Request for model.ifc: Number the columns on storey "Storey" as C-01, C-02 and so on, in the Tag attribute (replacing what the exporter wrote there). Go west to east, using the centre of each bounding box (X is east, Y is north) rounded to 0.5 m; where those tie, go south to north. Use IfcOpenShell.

First a look at what the model holds.

```python
import ifcopenshell
import ifcopenshell.util.element
import ifcopenshell.util.placement

model = ifcopenshell.open("model.ifc")
print(model.schema)
storey = next(s for s in model.by_type("IfcBuildingStorey") if s.Name == "Storey")
columns = [e for e in ifcopenshell.util.element.get_decomposition(storey) if e.is_a("IfcColumn")]
for e in sorted(columns, key=lambda e: e.id()):
    origin = ifcopenshell.util.placement.get_local_placement(e.ObjectPlacement)[:3, 3]
    print(e.id(), e.Tag, e.Name, origin.round(2) + 0.0, sep=" | ")
```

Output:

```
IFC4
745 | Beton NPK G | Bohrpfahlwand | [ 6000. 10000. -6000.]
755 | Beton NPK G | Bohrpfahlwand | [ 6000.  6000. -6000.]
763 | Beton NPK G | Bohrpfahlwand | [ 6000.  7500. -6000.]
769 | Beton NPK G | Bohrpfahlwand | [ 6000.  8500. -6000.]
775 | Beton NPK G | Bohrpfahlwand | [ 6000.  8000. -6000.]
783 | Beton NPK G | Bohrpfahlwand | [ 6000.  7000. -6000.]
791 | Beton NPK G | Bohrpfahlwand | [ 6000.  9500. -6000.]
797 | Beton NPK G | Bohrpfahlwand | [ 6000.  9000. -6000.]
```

```python
import ifcopenshell
import ifcopenshell.geom
import ifcopenshell.util.element
import ifcopenshell.util.shape

model = ifcopenshell.open("model.ifc")
settings = ifcopenshell.geom.settings()
settings.set("use-world-coords", True)


def centre(element):
    shape = ifcopenshell.geom.create_shape(settings, element)
    return ifcopenshell.util.shape.get_bbox_centroid(shape.geometry)


storey = next(s for s in model.by_type("IfcBuildingStorey") if s.Name == "Storey")
columns = [e for e in ifcopenshell.util.element.get_decomposition(storey) if e.is_a("IfcColumn")]

# Insertion points can sit at a corner or the storey origin, so sort by the geometry (in metres).
centres = {e: centre(e) for e in columns}
columns.sort(key=lambda e: (round(centres[e][0] / 0.5), centres[e][1]))

for i, e in enumerate(columns, start=1):
    number = f"C-{i:02d}"
    e.Tag = number
    print(e.id(), number)

model.write("model_edited.ifc")
```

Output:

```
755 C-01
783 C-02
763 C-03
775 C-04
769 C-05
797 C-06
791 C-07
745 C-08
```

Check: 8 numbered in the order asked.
